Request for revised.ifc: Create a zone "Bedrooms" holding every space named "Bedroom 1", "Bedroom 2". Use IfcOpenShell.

First a look at what the model holds.

```python
import ifcopenshell

model = ifcopenshell.open("revised.ifc")
print(model.schema)
seen = {}
for space in model.by_type("IfcSpace"):
    seen[space.LongName] = seen.get(space.LongName, 0) + 1
for name, count in sorted(seen.items(), key=str):
    print(count, "x", name)
print("zones:", [z.Name for z in model.by_type("IfcZone")][:20])
```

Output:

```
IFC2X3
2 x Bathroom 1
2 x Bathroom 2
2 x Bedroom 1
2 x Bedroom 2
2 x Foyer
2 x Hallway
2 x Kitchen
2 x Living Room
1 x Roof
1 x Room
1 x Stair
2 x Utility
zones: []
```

```python
import ifcopenshell
import ifcopenshell.api.group
import ifcopenshell.api.root

model = ifcopenshell.open("revised.ifc")

names = {"Bedroom 1", "Bedroom 2"}
spaces = [s for s in model.by_type("IfcSpace") if s.LongName in names]

zone = ifcopenshell.api.root.create_entity(model, ifc_class="IfcZone", name="Bedrooms")
ifcopenshell.api.group.assign_group(model, products=spaces, group=zone)
print(len(spaces), "spaces in", zone.Name)

model.write("revised-out.ifc")
```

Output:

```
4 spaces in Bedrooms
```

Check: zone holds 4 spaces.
